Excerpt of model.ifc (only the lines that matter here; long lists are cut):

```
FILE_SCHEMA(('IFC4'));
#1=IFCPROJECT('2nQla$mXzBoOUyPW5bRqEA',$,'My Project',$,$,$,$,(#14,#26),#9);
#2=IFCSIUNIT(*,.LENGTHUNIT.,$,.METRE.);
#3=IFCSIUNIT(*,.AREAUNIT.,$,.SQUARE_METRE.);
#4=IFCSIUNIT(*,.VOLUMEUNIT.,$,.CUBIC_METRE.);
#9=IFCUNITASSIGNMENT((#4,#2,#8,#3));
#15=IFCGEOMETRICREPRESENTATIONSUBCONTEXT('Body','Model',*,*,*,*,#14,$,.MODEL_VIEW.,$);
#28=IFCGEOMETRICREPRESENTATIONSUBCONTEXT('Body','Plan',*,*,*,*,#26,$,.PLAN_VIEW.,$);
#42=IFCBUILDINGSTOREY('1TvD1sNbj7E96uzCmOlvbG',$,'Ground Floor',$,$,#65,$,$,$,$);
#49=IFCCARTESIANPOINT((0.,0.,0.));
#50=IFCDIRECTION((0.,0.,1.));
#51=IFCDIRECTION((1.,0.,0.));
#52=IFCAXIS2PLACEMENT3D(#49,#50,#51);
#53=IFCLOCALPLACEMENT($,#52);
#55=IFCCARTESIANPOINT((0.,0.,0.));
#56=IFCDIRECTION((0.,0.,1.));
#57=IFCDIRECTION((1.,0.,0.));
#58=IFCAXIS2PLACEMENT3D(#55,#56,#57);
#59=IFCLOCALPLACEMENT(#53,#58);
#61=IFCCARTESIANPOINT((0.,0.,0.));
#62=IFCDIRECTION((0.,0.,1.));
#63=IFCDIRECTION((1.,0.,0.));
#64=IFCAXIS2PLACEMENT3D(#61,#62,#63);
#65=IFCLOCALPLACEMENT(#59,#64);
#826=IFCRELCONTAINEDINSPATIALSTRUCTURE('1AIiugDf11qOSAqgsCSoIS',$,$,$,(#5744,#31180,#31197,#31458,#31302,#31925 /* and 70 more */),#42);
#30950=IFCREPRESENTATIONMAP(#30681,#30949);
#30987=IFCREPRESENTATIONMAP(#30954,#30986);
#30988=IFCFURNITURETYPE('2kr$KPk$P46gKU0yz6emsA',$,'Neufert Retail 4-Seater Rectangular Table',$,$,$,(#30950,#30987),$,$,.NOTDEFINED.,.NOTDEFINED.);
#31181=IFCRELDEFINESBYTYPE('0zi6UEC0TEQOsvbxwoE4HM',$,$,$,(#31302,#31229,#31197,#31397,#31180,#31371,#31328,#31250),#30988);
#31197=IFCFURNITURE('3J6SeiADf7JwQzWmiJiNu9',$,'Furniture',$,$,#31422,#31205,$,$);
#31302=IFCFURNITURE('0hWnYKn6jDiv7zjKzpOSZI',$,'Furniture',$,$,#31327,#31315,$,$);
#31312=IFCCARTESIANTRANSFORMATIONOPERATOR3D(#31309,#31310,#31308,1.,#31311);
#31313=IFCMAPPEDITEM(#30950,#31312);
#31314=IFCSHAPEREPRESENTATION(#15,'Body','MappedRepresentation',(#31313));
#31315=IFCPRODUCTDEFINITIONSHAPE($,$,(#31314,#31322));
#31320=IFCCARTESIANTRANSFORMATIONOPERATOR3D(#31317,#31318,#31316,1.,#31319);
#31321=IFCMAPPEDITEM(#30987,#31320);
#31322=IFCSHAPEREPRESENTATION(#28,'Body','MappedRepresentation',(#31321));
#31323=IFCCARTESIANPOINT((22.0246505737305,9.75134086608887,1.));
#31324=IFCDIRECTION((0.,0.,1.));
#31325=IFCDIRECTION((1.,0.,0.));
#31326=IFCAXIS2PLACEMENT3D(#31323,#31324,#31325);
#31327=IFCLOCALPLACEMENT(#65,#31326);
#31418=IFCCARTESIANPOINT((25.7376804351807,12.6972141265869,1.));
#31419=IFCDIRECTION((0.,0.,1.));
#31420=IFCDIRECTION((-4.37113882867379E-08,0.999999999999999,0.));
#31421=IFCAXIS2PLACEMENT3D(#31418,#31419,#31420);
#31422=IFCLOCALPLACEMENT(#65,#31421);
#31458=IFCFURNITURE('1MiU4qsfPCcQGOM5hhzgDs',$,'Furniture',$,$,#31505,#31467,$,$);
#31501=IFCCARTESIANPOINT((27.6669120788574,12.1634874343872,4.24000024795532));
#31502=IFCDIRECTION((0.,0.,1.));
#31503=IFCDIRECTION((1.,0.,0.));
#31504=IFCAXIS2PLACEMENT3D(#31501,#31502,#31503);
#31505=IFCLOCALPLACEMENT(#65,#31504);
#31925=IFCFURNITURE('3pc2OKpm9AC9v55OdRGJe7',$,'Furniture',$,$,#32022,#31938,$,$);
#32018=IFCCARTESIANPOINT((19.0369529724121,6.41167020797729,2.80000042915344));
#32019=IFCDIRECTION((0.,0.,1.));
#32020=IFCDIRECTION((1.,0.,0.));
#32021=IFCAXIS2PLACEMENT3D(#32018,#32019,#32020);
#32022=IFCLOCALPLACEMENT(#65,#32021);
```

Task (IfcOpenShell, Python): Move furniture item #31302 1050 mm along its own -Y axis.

```python
import ifcopenshell
import ifcopenshell.api.geometry
import ifcopenshell.util.placement

model = ifcopenshell.open("model.ifc")

item = model.by_guid("0hWnYKn6jDiv7zjKzpOSZI")
matrix = ifcopenshell.util.placement.get_local_placement(item.ObjectPlacement)
matrix[:3, 3] -= matrix[:3, 1] * 1.05
ifcopenshell.api.geometry.edit_object_placement(model, product=item, matrix=matrix, is_si=False)

print(ifcopenshell.util.placement.get_local_placement(item.ObjectPlacement).round(3) + 0.0)

model.write("model_edited.ifc")
```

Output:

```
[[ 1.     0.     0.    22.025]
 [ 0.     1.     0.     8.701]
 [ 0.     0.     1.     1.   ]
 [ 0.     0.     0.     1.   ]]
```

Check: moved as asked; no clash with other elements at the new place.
